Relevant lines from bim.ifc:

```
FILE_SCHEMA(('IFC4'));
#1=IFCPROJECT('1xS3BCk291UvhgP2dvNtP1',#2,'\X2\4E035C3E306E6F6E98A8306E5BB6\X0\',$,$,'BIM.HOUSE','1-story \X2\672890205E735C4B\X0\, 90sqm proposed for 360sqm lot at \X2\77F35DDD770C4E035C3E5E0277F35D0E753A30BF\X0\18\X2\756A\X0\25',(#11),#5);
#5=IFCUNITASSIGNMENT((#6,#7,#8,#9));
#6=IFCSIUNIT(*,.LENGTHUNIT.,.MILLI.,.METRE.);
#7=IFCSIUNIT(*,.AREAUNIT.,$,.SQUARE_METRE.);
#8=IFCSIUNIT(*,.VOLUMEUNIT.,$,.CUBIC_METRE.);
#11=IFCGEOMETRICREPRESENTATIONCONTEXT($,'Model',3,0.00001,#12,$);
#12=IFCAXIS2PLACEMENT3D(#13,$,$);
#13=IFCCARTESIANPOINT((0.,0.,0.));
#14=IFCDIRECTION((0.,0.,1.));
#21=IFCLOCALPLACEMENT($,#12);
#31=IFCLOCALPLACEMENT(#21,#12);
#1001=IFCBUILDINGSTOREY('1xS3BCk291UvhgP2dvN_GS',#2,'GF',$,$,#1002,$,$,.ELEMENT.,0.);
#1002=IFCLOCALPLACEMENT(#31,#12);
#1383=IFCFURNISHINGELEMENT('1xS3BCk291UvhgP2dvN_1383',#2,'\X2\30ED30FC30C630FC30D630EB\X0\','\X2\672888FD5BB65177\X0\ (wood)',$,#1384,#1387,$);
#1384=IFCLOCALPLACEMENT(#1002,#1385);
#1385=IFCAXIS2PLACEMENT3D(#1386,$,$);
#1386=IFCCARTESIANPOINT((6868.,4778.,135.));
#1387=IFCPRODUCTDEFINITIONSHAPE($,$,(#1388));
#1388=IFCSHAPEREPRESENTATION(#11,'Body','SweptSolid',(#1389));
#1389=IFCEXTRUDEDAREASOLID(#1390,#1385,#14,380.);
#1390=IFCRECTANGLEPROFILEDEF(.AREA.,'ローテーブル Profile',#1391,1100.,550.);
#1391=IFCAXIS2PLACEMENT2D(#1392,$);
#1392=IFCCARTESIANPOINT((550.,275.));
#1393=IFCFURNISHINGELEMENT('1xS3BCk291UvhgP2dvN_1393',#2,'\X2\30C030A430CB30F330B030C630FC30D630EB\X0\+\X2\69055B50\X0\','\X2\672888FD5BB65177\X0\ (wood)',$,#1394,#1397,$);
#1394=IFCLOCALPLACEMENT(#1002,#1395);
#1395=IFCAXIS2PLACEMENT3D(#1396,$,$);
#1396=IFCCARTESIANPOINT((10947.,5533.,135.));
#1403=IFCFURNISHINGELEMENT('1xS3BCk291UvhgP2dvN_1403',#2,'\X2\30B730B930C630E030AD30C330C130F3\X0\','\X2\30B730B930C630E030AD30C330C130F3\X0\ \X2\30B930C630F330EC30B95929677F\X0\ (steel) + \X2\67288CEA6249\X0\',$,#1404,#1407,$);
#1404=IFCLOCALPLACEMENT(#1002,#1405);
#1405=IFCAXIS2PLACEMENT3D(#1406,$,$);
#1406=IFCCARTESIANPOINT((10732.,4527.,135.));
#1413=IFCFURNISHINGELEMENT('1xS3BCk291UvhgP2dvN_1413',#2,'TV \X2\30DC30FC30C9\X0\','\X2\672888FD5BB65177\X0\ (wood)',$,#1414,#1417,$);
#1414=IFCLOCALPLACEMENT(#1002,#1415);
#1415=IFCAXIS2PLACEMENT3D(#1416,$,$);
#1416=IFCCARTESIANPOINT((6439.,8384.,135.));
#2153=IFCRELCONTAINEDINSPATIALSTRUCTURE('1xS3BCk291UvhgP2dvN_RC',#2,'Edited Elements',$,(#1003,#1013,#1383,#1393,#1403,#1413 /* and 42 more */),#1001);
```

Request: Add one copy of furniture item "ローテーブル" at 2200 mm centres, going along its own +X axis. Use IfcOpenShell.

```python
import ifcopenshell
import ifcopenshell.api.geometry
import ifcopenshell.api.root
import ifcopenshell.util.element
import ifcopenshell.util.placement
import ifcopenshell.util.unit

model = ifcopenshell.open("bim.ifc")
unit_scale = ifcopenshell.util.unit.calculate_unit_scale(model)


def reuse_history(source, copy):
    """copy_class also copies each property set's owner history, people and application; keep the originals."""
    for rel in copy.IsDefinedBy:
        if rel.is_a("IfcRelDefinesByProperties") and (history := rel.RelatingPropertyDefinition.OwnerHistory):
            rel.RelatingPropertyDefinition.OwnerHistory = source.OwnerHistory
            ifcopenshell.util.element.remove_deep2(model, history)


source = model.by_id(1383)
base = ifcopenshell.util.placement.get_local_placement(source.ObjectPlacement)
step = base[:3, 0] * 2.2 / unit_scale

for i in range(1, 2):
    copy = ifcopenshell.api.root.copy_class(model, product=source)
    copy.Representation = ifcopenshell.util.element.copy_deep(
        model, source.Representation, exclude=["IfcGeometricRepresentationContext", "IfcRepresentationMap"]
    )
    reuse_history(source, copy)
    matrix = base.copy()
    matrix[:3, 3] += i * step
    print("added at", matrix[:3, 3].round(3) + 0.0)
    ifcopenshell.api.geometry.edit_object_placement(model, product=copy, matrix=matrix, is_si=False)

model.write("bim-out.ifc")
```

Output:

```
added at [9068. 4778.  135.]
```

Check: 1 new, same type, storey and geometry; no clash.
